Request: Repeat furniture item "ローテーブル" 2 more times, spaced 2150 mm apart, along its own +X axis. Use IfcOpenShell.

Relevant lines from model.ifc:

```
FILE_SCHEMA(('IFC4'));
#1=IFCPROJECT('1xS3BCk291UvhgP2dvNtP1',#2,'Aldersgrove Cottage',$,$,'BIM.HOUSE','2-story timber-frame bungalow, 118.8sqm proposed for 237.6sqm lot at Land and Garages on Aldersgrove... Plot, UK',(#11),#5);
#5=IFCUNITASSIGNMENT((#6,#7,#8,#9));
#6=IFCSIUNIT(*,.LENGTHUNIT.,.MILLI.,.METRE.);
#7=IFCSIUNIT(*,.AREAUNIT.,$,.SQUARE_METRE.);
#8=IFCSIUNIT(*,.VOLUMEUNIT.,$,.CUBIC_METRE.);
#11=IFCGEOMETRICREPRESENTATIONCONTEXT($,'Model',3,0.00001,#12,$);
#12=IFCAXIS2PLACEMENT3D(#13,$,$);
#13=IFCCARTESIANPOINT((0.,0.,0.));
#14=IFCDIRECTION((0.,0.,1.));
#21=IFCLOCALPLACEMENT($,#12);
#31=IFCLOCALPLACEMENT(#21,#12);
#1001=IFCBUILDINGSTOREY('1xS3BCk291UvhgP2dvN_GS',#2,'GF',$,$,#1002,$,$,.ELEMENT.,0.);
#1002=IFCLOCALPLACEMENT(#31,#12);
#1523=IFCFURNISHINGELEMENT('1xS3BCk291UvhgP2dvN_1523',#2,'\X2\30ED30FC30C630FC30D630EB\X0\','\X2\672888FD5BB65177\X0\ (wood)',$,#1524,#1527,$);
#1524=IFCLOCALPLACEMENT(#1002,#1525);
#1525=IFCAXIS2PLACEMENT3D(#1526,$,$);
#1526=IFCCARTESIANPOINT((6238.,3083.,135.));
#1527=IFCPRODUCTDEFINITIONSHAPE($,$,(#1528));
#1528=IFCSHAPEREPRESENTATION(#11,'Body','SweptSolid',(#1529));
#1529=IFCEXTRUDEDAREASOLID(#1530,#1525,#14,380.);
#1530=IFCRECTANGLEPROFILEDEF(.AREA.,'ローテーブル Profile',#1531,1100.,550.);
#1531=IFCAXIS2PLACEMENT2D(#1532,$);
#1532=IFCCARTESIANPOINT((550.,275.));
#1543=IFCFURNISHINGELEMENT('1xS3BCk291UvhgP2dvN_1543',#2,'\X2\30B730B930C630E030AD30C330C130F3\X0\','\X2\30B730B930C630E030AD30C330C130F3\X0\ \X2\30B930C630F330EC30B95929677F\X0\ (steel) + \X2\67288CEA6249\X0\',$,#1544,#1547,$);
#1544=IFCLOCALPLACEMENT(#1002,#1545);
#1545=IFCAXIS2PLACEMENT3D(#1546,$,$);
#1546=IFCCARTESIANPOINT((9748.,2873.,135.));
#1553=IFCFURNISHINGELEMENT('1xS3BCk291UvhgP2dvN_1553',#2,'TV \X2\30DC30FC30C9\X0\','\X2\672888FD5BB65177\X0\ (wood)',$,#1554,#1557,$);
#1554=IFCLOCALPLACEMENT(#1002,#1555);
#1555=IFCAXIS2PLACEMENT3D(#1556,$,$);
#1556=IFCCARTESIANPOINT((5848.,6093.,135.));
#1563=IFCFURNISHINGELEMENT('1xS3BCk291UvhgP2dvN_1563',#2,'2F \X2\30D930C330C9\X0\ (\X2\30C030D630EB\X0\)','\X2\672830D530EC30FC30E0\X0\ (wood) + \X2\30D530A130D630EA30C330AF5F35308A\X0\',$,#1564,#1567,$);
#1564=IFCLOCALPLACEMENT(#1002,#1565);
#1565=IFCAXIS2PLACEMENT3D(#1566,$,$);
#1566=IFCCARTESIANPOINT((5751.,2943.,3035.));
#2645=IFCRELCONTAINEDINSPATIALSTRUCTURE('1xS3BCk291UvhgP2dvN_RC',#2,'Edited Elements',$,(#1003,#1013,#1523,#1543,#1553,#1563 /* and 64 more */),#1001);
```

```python
import ifcopenshell
import ifcopenshell.api.geometry
import ifcopenshell.api.root
import ifcopenshell.util.element
import ifcopenshell.util.placement
import ifcopenshell.util.unit

model = ifcopenshell.open("model.ifc")
unit_scale = ifcopenshell.util.unit.calculate_unit_scale(model)


def reuse_history(source, copy):
    """copy_class also copies each property set's owner history, people and application; keep the originals."""
    for rel in copy.IsDefinedBy:
        if rel.is_a("IfcRelDefinesByProperties") and (history := rel.RelatingPropertyDefinition.OwnerHistory):
            rel.RelatingPropertyDefinition.OwnerHistory = source.OwnerHistory
            ifcopenshell.util.element.remove_deep2(model, history)


source = model.by_guid("1xS3BCk291UvhgP2dvN_1523")
base = ifcopenshell.util.placement.get_local_placement(source.ObjectPlacement)
step = base[:3, 0] * 2.15 / unit_scale

for i in range(1, 3):
    copy = ifcopenshell.api.root.copy_class(model, product=source)
    copy.Representation = ifcopenshell.util.element.copy_deep(
        model, source.Representation, exclude=["IfcGeometricRepresentationContext", "IfcRepresentationMap"]
    )
    reuse_history(source, copy)
    matrix = base.copy()
    matrix[:3, 3] += i * step
    print("added at", matrix[:3, 3].round(3) + 0.0)
    ifcopenshell.api.geometry.edit_object_placement(model, product=copy, matrix=matrix, is_si=False)

model.write("model_rev.ifc")
```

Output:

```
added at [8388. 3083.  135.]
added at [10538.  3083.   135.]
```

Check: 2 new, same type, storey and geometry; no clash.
